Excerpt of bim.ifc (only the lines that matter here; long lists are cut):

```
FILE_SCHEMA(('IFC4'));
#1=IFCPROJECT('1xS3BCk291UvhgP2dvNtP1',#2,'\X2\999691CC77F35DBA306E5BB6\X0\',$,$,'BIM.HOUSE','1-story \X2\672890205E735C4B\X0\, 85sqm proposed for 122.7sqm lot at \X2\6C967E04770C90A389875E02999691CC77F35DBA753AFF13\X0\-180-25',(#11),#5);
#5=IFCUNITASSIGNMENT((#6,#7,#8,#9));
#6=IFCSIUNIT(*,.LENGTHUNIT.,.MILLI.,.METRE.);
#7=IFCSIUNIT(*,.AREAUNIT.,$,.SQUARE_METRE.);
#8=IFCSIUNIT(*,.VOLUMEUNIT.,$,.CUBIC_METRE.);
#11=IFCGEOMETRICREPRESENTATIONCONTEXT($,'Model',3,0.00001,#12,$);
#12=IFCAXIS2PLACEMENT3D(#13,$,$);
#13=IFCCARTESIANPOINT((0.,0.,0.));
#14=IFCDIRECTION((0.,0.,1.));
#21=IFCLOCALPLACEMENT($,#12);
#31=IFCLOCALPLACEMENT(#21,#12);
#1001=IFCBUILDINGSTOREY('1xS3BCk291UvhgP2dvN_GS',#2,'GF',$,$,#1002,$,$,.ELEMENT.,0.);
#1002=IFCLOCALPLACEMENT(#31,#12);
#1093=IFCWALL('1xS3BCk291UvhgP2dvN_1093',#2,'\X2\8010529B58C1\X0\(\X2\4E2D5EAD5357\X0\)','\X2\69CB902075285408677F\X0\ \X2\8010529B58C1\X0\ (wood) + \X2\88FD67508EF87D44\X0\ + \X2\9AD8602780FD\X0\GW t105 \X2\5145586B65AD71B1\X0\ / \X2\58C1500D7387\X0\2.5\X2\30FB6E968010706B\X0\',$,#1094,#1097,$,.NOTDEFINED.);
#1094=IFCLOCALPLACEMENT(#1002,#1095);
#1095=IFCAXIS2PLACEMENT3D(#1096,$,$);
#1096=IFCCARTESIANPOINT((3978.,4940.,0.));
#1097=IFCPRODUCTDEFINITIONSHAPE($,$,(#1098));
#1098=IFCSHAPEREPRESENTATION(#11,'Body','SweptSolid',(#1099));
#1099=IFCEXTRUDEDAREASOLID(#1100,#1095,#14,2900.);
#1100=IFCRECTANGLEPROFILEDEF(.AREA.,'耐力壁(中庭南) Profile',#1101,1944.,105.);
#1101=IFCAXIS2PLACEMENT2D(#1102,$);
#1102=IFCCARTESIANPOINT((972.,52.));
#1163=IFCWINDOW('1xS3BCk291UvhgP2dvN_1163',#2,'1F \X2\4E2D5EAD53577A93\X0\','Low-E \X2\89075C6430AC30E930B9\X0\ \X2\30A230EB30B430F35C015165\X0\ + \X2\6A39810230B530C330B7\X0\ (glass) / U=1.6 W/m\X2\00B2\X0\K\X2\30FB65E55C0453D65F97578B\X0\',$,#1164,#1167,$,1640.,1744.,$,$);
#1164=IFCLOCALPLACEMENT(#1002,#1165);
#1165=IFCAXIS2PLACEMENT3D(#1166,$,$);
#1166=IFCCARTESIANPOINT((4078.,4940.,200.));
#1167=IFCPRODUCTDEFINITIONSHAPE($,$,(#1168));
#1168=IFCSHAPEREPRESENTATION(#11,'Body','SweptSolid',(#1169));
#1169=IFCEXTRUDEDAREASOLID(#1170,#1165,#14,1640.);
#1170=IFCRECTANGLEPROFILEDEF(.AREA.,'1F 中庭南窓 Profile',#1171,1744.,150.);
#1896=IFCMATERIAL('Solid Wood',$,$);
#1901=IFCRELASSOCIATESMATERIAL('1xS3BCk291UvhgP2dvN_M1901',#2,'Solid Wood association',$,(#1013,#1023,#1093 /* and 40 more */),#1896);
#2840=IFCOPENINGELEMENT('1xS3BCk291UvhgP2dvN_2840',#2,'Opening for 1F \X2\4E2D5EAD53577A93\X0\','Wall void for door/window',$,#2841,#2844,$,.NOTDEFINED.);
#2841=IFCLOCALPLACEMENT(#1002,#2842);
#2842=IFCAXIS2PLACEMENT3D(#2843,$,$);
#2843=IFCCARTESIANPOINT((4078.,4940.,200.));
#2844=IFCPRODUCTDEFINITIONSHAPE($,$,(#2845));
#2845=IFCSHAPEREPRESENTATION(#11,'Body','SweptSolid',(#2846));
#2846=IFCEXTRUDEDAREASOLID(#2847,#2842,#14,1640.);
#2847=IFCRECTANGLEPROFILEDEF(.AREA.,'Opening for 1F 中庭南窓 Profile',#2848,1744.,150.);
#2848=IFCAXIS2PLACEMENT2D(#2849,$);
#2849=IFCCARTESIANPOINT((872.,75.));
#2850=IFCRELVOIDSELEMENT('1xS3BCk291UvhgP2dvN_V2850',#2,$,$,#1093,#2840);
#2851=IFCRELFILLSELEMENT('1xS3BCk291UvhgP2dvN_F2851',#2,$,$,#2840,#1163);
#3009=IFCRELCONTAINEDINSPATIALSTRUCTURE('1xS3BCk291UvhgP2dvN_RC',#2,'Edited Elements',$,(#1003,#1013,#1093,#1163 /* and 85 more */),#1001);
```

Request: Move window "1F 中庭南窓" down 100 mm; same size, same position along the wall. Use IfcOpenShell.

```python
import numpy as np
import ifcopenshell
import ifcopenshell.api.geometry
import ifcopenshell.util.placement
import ifcopenshell.util.unit

model = ifcopenshell.open("bim.ifc")
unit_scale = ifcopenshell.util.unit.calculate_unit_scale(model)

window = model.by_guid("1xS3BCk291UvhgP2dvN_1163")
opening = window.FillsVoids[0].RelatingOpeningElement
dz = -100.0

shift = np.array([0.0, 0.0, dz])
# The window is not placed relative to its opening, so move both.
for product in (opening, window):
    matrix = ifcopenshell.util.placement.get_local_placement(product.ObjectPlacement)
    matrix[:3, 3] += shift
    ifcopenshell.api.geometry.edit_object_placement(model, product=product, matrix=matrix, is_si=False)

print(f"moved by {dz * unit_scale:+.3f} m")

model.write("bim-out.ifc")
```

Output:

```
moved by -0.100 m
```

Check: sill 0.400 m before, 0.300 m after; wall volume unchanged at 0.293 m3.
